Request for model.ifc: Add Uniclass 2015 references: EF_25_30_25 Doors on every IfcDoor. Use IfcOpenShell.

First a look at what the model holds.

```python
import ifcopenshell

model = ifcopenshell.open("model.ifc")
print(model.schema)
print("classifications:", [c.Name for c in model.by_type("IfcClassification")])
for ifc_class in ("IfcDoor", "IfcRoof", "IfcStair", "IfcWall", "IfcWindow"):
    print(ifc_class, len(model.by_type(ifc_class)))
```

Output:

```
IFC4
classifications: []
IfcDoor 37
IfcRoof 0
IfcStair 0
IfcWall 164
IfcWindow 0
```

```python
import ifcopenshell
import ifcopenshell.api.classification

model = ifcopenshell.open("model.ifc")

system = ifcopenshell.api.classification.add_classification(model, classification="Uniclass 2015")

codes = {
    "IfcDoor": ("EF_25_30_25", "Doors"),
}
for ifc_class, (code, name) in codes.items():
    products = model.by_type(ifc_class)
    ifcopenshell.api.classification.add_reference(
        model, products=products, classification=system, identification=code, name=name
    )
    print(code, len(products))

model.write("model_rev.ifc")
```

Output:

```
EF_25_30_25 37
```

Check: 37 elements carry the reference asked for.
